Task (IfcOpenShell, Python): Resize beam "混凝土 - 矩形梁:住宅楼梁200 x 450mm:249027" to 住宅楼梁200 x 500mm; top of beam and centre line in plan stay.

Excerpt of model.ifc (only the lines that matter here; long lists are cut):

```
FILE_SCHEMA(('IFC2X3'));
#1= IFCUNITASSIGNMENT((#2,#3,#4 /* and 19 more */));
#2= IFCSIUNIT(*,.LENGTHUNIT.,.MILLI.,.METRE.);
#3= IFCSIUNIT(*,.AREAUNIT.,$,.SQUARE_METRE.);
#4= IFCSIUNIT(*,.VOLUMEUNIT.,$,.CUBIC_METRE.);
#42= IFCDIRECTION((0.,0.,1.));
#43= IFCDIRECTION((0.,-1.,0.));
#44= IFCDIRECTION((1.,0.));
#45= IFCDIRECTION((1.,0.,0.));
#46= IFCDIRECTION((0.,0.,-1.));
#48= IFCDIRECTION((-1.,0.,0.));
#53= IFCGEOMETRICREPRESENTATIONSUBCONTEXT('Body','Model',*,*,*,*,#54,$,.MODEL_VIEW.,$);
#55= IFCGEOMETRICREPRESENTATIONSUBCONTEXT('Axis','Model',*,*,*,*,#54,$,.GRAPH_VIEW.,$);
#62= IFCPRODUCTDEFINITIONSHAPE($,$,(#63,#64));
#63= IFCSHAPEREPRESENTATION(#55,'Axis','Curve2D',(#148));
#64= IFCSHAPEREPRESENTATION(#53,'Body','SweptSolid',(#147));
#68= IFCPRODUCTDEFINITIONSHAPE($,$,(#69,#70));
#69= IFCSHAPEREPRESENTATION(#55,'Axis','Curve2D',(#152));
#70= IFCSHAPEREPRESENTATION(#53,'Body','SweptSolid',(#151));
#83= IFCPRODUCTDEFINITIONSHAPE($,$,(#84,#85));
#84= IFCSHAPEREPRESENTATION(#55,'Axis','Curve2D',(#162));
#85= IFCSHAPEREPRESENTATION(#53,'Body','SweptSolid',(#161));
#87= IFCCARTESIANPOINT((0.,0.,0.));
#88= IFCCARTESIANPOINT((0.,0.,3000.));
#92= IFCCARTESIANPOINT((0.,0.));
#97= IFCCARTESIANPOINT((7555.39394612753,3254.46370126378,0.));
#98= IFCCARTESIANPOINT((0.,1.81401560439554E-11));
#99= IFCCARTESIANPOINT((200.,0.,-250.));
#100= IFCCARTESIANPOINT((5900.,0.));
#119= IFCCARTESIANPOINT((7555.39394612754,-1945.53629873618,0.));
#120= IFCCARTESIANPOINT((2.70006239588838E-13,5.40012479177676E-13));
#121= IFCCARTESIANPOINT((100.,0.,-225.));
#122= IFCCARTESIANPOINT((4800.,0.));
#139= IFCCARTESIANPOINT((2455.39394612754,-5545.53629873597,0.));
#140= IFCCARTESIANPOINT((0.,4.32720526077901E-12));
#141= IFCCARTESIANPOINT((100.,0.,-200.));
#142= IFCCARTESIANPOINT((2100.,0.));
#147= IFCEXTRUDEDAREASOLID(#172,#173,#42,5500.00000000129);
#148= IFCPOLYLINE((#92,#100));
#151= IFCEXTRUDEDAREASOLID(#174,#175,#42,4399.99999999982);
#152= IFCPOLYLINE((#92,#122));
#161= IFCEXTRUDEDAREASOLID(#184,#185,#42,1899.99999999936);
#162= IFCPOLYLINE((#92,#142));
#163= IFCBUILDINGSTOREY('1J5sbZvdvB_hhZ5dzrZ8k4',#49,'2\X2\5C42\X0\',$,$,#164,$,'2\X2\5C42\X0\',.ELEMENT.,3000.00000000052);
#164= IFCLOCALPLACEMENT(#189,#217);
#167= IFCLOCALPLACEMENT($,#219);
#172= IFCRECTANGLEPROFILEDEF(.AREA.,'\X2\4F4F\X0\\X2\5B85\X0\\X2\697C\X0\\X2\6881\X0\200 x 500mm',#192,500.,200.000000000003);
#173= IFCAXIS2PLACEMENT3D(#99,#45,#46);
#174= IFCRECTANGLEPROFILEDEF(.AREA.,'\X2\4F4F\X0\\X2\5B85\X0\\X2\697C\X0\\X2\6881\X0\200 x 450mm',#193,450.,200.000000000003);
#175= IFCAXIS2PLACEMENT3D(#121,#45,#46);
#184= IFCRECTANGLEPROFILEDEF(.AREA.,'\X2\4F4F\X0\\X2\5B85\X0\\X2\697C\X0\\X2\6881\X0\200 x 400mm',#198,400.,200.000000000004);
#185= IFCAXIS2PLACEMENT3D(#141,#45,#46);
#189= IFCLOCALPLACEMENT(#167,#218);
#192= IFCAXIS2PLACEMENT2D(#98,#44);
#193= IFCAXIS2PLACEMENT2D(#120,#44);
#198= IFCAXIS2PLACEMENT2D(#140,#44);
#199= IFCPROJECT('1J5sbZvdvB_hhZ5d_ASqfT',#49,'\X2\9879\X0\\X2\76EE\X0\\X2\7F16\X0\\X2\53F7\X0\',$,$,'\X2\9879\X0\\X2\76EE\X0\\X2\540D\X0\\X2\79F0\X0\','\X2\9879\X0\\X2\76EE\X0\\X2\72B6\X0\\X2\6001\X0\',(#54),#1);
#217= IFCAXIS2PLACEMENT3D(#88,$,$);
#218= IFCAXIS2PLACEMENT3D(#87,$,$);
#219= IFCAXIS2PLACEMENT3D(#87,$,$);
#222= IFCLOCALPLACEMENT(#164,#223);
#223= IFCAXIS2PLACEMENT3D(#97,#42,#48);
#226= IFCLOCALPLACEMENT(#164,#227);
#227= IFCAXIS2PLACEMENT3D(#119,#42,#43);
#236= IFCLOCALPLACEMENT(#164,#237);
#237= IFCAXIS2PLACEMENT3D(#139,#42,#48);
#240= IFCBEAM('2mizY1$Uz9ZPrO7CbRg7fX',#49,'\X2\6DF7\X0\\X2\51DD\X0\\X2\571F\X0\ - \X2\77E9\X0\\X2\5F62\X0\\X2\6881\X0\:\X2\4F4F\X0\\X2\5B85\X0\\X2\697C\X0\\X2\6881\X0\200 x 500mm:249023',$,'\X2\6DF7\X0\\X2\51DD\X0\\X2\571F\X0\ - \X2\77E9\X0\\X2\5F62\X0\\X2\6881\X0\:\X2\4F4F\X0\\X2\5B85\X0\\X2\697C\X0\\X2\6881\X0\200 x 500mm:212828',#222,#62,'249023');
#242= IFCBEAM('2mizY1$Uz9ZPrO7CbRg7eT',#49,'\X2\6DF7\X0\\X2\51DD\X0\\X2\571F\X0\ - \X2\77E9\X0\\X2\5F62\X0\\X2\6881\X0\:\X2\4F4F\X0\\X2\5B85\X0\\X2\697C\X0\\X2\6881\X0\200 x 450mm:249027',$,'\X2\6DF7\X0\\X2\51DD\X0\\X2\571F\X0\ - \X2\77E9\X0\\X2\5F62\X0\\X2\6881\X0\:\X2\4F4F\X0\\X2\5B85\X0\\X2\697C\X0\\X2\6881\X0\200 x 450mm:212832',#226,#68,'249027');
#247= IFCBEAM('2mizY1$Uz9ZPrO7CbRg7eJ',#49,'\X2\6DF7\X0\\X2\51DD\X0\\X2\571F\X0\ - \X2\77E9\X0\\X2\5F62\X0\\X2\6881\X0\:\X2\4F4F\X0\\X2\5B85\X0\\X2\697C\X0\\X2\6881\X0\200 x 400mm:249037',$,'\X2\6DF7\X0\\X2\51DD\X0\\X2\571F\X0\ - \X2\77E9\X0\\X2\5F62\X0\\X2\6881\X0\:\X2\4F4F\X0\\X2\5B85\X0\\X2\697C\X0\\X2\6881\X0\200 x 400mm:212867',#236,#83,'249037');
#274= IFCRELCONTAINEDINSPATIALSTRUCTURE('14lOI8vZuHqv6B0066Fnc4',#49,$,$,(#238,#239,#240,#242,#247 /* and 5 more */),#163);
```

```python
import ifcopenshell
import ifcopenshell.util.element
import ifcopenshell.util.representation

model = ifcopenshell.open("model.ifc")

member = model.by_guid("2mizY1$Uz9ZPrO7CbRg7eT")
source = next(p for p in model.by_type("IfcRectangleProfileDef") if p.ProfileName == "住宅楼梁200 x 500mm")

body = ifcopenshell.util.representation.get_representation(member, "Model", "Body")
solid = body.Items[0]
old_profile = solid.SweptArea

# Copy the section's sizes but keep this member's own profile position.
profile = ifcopenshell.util.element.copy(model, source)
# Profiles are centred, so shift by half the change in depth to hold the top.
shift = (old_profile.XDim - profile.XDim) / 2
x, y = old_profile.Position.Location.Coordinates
up = (-1.0, 0.0)  # upwards, in the solid's own plane
location = model.createIfcCartesianPoint((x + up[0] * shift, y + up[1] * shift))
profile.Position = model.createIfcAxis2Placement2D(location, old_profile.Position.RefDirection)
solid.SweptArea = profile
if not model.get_total_inverses(old_profile):
    ifcopenshell.util.element.remove_deep2(model, old_profile)
member.Name = member.Name.replace("住宅楼梁200 x 450mm", "住宅楼梁200 x 500mm")
member.ObjectType = member.ObjectType.replace("住宅楼梁200 x 450mm", "住宅楼梁200 x 500mm")

print(solid.SweptArea)

model.write("model_v2.ifc")
```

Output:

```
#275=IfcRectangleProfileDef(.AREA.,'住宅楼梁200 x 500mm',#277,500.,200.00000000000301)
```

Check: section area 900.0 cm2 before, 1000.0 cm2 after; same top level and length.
